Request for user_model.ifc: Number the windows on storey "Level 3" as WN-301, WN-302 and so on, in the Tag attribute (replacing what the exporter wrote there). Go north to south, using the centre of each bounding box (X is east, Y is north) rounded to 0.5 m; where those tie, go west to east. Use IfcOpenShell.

First a look at what the model holds.

```python
import ifcopenshell
import ifcopenshell.util.element
import ifcopenshell.util.placement

model = ifcopenshell.open("user_model.ifc")
print(model.schema)
storey = next(s for s in model.by_type("IfcBuildingStorey") if s.Name == "Level 3")
windows = [e for e in ifcopenshell.util.element.get_decomposition(storey) if e.is_a("IfcWindow")]
for e in sorted(windows, key=lambda e: e.id()):
    origin = ifcopenshell.util.placement.get_local_placement(e.ObjectPlacement)[:3, 3]
    print(e.id(), e.Tag, e.Name, origin.round(2) + 0.0, sep=" | ")
```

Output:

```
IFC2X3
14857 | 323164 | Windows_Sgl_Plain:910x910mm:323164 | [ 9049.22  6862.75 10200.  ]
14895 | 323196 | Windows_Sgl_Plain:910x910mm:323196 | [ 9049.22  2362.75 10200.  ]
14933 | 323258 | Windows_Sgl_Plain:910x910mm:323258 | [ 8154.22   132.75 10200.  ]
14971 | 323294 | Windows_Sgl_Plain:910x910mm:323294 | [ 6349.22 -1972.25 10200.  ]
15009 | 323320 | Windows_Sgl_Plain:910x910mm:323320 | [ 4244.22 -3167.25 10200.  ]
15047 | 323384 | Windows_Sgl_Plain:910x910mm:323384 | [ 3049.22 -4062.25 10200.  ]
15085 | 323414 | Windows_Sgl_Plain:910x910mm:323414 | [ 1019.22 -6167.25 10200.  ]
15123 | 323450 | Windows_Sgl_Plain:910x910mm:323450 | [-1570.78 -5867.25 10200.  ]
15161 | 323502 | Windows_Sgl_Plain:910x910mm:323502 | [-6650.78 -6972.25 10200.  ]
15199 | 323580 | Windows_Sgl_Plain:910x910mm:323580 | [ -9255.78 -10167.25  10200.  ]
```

```python
import ifcopenshell
import ifcopenshell.geom
import ifcopenshell.util.element
import ifcopenshell.util.shape

model = ifcopenshell.open("user_model.ifc")
settings = ifcopenshell.geom.settings()
settings.set("use-world-coords", True)


def centre(element):
    shape = ifcopenshell.geom.create_shape(settings, element)
    return ifcopenshell.util.shape.get_bbox_centroid(shape.geometry)


storey = next(s for s in model.by_type("IfcBuildingStorey") if s.Name == "Level 3")
windows = [e for e in ifcopenshell.util.element.get_decomposition(storey) if e.is_a("IfcWindow")]

# Insertion points can sit at a corner or the storey origin, so sort by the geometry (in metres).
centres = {e: centre(e) for e in windows}
windows.sort(key=lambda e: (-round(centres[e][1] / 0.5), centres[e][0]))

for i, e in enumerate(windows, start=1):
    number = f"WN-3{i:02d}"
    e.Tag = number
    print(e.id(), number)

model.write("user_model_rev.ifc")
```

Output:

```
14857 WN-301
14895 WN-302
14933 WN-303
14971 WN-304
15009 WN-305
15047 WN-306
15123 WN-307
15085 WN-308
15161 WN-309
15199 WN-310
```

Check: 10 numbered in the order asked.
